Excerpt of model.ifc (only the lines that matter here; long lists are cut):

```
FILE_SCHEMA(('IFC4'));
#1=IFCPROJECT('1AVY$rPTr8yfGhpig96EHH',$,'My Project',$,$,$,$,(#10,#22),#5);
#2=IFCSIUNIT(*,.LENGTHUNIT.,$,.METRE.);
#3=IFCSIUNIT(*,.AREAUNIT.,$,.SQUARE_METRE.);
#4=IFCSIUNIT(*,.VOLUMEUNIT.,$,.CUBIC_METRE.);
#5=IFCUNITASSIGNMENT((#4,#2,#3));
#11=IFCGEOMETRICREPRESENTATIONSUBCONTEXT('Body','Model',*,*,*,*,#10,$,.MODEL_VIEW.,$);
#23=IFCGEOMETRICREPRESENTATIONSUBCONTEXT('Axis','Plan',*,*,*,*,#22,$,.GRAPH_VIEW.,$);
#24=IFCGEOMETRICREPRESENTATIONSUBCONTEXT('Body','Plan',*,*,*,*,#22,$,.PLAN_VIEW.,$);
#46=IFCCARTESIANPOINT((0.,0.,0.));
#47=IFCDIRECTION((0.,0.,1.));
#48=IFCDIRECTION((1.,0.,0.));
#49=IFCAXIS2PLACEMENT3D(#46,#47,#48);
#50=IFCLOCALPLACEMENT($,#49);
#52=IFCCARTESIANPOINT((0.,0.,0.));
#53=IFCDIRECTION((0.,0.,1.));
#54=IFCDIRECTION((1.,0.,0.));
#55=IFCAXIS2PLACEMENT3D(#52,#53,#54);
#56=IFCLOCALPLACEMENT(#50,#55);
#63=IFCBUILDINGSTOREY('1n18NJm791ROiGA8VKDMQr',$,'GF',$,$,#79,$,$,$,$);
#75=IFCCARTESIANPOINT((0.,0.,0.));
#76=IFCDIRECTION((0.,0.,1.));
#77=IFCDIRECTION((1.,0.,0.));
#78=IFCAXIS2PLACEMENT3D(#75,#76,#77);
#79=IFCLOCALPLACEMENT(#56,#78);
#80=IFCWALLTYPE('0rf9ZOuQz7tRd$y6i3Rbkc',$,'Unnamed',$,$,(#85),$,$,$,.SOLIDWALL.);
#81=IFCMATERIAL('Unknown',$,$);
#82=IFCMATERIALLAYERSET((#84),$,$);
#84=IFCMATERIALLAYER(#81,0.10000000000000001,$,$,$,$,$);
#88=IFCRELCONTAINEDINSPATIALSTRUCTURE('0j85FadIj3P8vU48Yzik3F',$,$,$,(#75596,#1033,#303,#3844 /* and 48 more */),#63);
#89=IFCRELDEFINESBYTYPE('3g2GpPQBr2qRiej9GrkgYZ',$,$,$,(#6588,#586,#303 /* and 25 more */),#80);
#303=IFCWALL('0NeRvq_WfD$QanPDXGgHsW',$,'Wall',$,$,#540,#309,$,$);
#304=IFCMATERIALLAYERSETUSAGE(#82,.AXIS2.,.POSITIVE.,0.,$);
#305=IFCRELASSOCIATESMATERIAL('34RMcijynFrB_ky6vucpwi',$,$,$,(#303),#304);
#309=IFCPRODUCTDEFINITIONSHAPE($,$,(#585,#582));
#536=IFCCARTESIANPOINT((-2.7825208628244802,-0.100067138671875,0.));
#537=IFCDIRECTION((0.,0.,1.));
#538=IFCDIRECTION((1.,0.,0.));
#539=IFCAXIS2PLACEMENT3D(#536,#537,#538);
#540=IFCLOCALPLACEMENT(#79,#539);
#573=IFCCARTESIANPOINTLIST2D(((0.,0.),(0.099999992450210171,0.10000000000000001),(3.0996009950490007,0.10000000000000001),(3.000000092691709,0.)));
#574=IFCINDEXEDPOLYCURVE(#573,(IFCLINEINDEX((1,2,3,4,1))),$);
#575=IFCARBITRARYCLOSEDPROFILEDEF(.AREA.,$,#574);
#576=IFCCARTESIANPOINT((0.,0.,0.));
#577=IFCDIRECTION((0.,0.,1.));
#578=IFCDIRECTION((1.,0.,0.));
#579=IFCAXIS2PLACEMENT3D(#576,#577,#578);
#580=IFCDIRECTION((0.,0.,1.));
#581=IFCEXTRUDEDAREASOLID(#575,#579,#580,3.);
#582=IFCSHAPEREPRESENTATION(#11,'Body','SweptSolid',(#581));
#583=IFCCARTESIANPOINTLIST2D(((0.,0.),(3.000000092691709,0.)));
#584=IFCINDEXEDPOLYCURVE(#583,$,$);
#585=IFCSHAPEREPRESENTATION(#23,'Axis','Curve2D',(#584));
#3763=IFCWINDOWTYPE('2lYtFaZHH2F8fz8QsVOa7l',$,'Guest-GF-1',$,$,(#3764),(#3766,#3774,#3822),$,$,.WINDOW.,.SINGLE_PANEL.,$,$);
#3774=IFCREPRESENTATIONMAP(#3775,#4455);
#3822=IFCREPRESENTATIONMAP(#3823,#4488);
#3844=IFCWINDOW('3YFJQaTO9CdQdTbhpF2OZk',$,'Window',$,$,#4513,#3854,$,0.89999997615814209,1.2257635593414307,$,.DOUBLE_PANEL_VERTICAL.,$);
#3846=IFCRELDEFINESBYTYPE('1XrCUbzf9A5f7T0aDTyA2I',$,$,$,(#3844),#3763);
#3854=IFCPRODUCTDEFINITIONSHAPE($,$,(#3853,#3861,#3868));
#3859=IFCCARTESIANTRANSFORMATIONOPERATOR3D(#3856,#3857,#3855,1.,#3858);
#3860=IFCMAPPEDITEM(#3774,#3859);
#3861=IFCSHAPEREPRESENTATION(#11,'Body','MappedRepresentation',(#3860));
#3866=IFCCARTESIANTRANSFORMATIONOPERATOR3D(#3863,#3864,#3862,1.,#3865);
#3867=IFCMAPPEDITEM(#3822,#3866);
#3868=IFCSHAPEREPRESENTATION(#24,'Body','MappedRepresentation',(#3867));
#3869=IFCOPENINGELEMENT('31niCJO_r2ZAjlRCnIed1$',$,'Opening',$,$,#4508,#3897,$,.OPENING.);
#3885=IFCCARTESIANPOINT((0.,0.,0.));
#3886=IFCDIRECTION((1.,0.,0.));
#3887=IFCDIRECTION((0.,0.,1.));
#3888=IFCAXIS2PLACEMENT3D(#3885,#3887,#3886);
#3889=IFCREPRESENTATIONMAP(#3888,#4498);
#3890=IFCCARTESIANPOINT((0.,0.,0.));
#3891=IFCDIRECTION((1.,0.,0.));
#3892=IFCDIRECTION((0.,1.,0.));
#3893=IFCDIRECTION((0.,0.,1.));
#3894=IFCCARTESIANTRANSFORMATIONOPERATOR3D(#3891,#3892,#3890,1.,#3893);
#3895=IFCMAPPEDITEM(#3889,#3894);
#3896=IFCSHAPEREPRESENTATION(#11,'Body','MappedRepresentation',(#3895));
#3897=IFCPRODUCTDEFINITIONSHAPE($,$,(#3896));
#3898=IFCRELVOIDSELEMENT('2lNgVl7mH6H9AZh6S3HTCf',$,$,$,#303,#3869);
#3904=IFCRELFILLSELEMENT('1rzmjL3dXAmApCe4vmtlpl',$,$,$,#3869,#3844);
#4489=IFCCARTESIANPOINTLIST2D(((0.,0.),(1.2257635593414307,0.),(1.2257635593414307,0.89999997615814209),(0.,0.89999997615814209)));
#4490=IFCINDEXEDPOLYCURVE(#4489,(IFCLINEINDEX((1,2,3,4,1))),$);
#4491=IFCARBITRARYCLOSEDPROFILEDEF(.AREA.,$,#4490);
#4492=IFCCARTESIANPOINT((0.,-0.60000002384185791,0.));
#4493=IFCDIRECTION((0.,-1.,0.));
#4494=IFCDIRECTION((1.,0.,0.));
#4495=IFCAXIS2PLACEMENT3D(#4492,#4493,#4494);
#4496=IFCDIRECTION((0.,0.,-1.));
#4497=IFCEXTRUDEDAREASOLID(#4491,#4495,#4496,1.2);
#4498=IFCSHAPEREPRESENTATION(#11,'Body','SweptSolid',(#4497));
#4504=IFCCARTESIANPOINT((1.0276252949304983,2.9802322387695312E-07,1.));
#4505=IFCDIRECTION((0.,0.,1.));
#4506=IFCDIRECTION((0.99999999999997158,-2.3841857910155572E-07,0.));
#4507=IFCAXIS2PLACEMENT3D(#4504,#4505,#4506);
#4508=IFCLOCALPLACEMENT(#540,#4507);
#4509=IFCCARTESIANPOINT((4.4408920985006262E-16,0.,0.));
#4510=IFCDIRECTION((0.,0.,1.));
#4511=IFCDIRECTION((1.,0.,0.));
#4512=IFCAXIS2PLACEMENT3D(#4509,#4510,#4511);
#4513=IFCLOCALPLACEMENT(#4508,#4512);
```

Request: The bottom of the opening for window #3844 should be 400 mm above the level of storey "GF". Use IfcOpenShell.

```python
import numpy as np
import ifcopenshell
import ifcopenshell.api.geometry
import ifcopenshell.geom
import ifcopenshell.util.element
import ifcopenshell.util.placement
import ifcopenshell.util.shape
import ifcopenshell.util.unit

model = ifcopenshell.open("model.ifc")
unit_scale = ifcopenshell.util.unit.calculate_unit_scale(model)

window = model.by_guid("3YFJQaTO9CdQdTbhpF2OZk")
opening = window.FillsVoids[0].RelatingOpeningElement
storey = ifcopenshell.util.element.get_container(window, ifc_class="IfcBuildingStorey")
level = ifcopenshell.util.placement.get_local_placement(storey.ObjectPlacement)[2, 3]

# The opening's origin need not be at the sill, so measure its lowest point.
shape = ifcopenshell.geom.create_shape(ifcopenshell.geom.settings(), opening)
bottom = ifcopenshell.util.shape.get_shape_bottom_elevation(shape, shape.geometry) / unit_scale
dz = level + 0.4 / unit_scale - bottom

shift = np.array([0.0, 0.0, dz])
# The window is placed relative to its opening, so it follows when the opening moves.
matrix = ifcopenshell.util.placement.get_local_placement(opening.ObjectPlacement)
matrix[:3, 3] += shift
ifcopenshell.api.geometry.edit_object_placement(
    model, product=opening, matrix=matrix, is_si=False, should_transform_children=True
)

print(f"moved by {dz * unit_scale:+.3f} m")

model.write("model_rev.ifc")
```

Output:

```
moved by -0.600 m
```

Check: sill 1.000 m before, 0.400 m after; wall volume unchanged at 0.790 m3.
